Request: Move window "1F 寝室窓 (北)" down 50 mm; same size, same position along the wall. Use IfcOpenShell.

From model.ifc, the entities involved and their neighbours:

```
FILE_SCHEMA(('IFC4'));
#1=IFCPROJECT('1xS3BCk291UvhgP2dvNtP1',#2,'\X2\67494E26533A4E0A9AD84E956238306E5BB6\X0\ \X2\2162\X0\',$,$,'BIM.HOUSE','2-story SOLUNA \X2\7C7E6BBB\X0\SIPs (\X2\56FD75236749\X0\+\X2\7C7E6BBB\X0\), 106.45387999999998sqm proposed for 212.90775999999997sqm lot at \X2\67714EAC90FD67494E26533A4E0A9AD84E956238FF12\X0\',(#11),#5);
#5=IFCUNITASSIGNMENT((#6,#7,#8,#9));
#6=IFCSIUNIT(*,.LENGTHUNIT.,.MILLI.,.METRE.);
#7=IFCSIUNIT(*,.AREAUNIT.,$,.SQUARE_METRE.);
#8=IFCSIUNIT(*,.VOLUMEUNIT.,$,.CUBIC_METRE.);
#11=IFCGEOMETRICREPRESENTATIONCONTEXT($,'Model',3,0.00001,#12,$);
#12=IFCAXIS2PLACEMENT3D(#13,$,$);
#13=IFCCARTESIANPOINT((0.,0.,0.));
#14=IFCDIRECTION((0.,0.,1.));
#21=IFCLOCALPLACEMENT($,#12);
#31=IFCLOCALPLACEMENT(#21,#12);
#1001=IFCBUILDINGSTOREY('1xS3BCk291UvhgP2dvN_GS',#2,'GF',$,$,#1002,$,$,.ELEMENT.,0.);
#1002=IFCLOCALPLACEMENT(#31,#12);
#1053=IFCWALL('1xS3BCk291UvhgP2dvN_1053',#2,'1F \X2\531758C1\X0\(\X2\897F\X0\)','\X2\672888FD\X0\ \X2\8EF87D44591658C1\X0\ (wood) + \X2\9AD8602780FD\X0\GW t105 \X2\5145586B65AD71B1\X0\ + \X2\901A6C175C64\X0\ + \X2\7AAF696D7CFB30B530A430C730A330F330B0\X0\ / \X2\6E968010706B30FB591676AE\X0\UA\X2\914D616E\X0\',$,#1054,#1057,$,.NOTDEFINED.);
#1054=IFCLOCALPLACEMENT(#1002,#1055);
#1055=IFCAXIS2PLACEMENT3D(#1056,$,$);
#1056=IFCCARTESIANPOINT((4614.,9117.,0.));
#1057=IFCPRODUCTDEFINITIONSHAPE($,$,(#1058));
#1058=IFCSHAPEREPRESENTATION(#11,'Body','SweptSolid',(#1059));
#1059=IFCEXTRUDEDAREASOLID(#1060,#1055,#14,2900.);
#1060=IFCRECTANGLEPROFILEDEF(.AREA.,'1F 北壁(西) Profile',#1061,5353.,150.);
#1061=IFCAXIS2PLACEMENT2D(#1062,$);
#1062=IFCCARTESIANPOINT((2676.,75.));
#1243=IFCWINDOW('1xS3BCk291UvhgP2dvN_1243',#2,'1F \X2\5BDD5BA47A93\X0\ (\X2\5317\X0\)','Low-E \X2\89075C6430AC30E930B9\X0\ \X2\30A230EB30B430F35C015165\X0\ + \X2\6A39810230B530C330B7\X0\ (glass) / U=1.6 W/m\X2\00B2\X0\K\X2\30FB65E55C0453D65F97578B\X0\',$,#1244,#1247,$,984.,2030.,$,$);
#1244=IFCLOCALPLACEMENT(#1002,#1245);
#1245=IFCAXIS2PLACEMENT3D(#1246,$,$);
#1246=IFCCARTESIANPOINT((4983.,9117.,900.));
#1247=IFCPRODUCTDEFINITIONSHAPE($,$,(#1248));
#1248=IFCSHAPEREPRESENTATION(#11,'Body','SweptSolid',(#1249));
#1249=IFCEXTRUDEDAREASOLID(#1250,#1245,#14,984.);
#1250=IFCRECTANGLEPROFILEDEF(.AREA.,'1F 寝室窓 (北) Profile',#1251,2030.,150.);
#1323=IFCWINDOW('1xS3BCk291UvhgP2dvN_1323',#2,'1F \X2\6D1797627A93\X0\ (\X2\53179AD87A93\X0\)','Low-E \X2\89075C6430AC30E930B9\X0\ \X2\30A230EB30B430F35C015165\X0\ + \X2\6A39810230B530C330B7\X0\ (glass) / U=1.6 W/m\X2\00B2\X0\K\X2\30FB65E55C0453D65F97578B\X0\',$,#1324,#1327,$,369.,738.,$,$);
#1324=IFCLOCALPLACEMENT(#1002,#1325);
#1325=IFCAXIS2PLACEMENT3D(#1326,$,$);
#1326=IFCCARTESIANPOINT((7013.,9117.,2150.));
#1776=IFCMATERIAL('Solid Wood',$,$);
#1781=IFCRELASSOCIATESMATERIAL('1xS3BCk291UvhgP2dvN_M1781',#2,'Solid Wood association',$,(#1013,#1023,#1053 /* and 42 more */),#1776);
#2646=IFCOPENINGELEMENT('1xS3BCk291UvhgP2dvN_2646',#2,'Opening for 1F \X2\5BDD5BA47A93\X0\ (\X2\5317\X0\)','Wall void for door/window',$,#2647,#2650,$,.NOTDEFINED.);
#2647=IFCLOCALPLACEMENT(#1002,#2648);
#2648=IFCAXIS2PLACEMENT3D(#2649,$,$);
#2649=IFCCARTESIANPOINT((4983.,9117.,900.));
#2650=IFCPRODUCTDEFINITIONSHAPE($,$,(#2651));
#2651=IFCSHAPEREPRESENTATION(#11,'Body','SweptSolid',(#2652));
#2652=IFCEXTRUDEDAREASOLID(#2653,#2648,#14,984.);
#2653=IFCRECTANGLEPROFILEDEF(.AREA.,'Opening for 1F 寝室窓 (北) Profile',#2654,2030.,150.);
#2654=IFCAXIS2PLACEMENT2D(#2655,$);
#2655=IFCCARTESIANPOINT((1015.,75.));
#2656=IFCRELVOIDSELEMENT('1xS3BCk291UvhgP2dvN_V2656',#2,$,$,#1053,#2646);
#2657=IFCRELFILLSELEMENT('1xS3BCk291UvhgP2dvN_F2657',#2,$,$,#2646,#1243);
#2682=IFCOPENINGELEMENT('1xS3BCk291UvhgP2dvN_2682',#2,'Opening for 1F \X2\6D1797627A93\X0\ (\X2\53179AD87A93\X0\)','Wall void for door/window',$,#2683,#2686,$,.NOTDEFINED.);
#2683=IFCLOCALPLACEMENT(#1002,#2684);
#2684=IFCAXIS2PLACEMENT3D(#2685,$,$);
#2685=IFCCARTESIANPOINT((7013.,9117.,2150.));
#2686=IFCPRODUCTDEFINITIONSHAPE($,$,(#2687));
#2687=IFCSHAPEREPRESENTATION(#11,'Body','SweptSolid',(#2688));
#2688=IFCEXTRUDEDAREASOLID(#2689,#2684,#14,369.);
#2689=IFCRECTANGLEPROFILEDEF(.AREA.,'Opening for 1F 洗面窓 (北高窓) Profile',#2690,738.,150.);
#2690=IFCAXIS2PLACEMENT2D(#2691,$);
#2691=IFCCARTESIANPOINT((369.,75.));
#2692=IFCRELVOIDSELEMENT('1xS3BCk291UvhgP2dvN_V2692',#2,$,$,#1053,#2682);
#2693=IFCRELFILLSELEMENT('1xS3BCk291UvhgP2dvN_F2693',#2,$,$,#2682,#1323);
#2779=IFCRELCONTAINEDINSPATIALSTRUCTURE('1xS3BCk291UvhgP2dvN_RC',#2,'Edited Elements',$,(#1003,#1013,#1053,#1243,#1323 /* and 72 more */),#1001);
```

```python
import numpy as np
import ifcopenshell
import ifcopenshell.api.geometry
import ifcopenshell.util.placement
import ifcopenshell.util.unit

model = ifcopenshell.open("model.ifc")
unit_scale = ifcopenshell.util.unit.calculate_unit_scale(model)

window = model.by_guid("1xS3BCk291UvhgP2dvN_1243")
opening = window.FillsVoids[0].RelatingOpeningElement
dz = -50.0

shift = np.array([0.0, 0.0, dz])
# The window is not placed relative to its opening, so move both.
for product in (opening, window):
    matrix = ifcopenshell.util.placement.get_local_placement(product.ObjectPlacement)
    matrix[:3, 3] += shift
    ifcopenshell.api.geometry.edit_object_placement(model, product=product, matrix=matrix, is_si=False)

print(f"moved by {dz * unit_scale:+.3f} m")

model.write("model_edited.ifc")
```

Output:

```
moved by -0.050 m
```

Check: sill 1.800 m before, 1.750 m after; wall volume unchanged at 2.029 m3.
